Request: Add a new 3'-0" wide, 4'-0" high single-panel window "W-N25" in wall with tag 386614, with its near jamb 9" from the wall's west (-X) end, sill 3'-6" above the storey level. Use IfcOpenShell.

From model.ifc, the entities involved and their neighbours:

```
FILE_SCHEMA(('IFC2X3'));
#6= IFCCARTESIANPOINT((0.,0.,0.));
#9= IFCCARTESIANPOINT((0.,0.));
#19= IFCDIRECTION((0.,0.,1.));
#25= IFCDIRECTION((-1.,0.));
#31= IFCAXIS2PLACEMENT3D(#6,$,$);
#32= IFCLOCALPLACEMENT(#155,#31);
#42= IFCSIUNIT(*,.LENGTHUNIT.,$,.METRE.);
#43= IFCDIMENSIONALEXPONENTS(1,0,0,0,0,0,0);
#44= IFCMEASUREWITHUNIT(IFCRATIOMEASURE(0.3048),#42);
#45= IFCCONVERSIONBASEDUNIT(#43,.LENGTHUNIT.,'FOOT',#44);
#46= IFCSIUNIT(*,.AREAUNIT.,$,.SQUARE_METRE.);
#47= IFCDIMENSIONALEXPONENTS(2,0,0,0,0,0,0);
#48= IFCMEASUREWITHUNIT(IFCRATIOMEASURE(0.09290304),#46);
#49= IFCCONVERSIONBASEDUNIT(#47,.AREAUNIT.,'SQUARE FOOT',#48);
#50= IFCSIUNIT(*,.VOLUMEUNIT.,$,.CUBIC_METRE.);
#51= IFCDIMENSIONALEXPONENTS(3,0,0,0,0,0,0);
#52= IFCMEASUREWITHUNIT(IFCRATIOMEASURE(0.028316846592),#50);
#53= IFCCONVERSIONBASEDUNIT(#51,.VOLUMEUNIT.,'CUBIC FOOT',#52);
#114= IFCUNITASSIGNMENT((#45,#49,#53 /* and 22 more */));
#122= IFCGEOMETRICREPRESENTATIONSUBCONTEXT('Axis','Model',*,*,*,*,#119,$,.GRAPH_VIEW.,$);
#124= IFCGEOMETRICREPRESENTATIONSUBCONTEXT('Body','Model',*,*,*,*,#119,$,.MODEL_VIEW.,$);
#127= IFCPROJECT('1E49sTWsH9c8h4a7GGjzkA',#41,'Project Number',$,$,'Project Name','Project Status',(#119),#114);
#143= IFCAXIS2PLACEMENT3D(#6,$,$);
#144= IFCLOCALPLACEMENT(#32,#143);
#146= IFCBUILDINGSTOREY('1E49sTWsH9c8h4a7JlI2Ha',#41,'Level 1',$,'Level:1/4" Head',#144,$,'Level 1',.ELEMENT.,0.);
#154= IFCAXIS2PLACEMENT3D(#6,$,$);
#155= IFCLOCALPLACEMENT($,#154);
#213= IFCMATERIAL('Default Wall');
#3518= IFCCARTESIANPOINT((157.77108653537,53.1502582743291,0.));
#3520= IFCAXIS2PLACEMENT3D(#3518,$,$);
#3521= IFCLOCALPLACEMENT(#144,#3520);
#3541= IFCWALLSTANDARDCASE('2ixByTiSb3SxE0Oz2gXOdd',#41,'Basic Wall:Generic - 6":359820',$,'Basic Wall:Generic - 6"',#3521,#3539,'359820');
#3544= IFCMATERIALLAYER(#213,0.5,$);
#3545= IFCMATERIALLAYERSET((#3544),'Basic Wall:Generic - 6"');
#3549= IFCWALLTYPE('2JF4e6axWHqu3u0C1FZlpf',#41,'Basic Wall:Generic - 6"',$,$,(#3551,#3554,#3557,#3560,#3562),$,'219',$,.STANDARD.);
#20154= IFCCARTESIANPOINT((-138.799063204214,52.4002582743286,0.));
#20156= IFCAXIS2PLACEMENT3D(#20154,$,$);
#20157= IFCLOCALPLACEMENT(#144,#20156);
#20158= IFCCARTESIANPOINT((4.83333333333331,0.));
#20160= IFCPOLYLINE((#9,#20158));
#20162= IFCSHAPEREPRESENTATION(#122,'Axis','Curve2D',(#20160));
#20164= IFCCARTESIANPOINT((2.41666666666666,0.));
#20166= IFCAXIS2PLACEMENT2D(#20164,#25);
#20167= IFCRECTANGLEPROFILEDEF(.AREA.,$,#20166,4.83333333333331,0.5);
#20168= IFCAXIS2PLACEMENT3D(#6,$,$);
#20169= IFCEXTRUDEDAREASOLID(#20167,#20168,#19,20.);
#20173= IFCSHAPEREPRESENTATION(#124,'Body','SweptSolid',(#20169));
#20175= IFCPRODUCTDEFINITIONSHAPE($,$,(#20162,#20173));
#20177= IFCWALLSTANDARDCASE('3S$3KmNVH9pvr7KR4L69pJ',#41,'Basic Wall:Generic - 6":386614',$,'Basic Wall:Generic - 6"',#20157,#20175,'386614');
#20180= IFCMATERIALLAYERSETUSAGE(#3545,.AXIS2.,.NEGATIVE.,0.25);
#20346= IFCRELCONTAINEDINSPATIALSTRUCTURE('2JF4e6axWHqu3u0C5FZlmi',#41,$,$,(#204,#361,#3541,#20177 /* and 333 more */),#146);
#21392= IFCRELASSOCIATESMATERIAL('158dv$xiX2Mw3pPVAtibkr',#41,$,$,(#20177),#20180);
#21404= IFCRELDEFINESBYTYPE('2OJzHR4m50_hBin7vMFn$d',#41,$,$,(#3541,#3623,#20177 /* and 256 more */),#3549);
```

```python
import numpy as np
import ifcopenshell
import ifcopenshell.api.feature
import ifcopenshell.api.geometry
import ifcopenshell.api.root
import ifcopenshell.api.spatial
import ifcopenshell.api.type
import ifcopenshell.geom
import ifcopenshell.util.element
import ifcopenshell.util.placement
import ifcopenshell.util.representation
import ifcopenshell.util.shape
import ifcopenshell.util.unit

model = ifcopenshell.open("model.ifc")
unit_scale = ifcopenshell.util.unit.calculate_unit_scale(model)
settings = ifcopenshell.geom.settings()


def volume(element):
    """Net volume in cubic metres, openings subtracted."""
    shape = ifcopenshell.geom.create_shape(settings, element)
    return ifcopenshell.util.shape.get_volume(shape.geometry)


wall = model.by_guid("3S$3KmNVH9pvr7KR4L69pJ")
storey = ifcopenshell.util.element.get_container(wall, ifc_class="IfcBuildingStorey")
context = ifcopenshell.util.representation.get_context(model, "Model", "Body", "MODEL_VIEW")
before = volume(wall)

width, height, from_end, sill = 0.9144, 1.2192, 0.2286, 1.0668  # metres

# The wall runs along its own X axis, and the end named is its -X end.
wall_shape = ifcopenshell.geom.create_shape(settings, wall)
x, y, z = ifcopenshell.util.shape.get_vertices(wall_shape.geometry).T
start = x.min() + from_end
face, thickness = float(y.min()), float(y.max() - y.min())
wall_matrix = ifcopenshell.util.placement.get_local_placement(wall.ObjectPlacement)
level = ifcopenshell.util.placement.get_local_placement(storey.ObjectPlacement)[2, 3]


def in_wall(x, y):
    """Placement at x, y metres in the wall's axes, at sill height."""
    matrix = wall_matrix.copy()
    matrix[:, 3] = wall_matrix @ np.array([x / unit_scale, y / unit_scale, 0.0, 1.0])
    matrix[2, 3] = level + sill / unit_scale
    return matrix


# Opening: a box that overshoots both wall faces by 50 mm.
opening = ifcopenshell.api.root.create_entity(model, ifc_class="IfcOpeningElement")
box = ifcopenshell.api.geometry.add_wall_representation(
    model, context=context, length=width, height=height, thickness=thickness + 0.1
)
ifcopenshell.api.geometry.assign_representation(model, product=opening, representation=box)
ifcopenshell.api.geometry.edit_object_placement(model, product=opening, matrix=in_wall(start, face - 0.05), is_si=False)
ifcopenshell.api.feature.add_feature(model, feature=opening, element=wall)

window = ifcopenshell.api.root.create_entity(model, ifc_class="IfcWindow", name="W-N25")
window.OverallWidth, window.OverallHeight = width / unit_scale, height / unit_scale
body = ifcopenshell.api.geometry.add_window_representation(
    model,
    context=context,
    overall_width=window.OverallWidth,
    overall_height=window.OverallHeight,
    partition_type="SINGLE_PANEL",
)
ifcopenshell.api.geometry.assign_representation(model, product=window, representation=body)
ifcopenshell.api.spatial.assign_container(model, products=[window], relating_structure=storey)
fills = ifcopenshell.api.feature.add_filling(model, opening=opening, element=window)
fills.OwnerHistory = window.OwnerHistory  # required in IFC2X3

# IFC2X3 keeps the operation on the window style.
style = ifcopenshell.api.root.create_entity(model, ifc_class="IfcWindowStyle", name="W-N25")
style.OperationType, style.ConstructionType = "SINGLE_PANEL", "NOTDEFINED"
style.ParameterTakesPrecedence = style.Sizeable = False
ifcopenshell.api.type.assign_type(model, related_objects=[window], relating_type=style)

# Centre the window in the wall's thickness.
ifcopenshell.api.geometry.edit_object_placement(model, product=window, matrix=in_wall(start, face), is_si=False)
window_shape = ifcopenshell.geom.create_shape(settings, window)
depth = ifcopenshell.util.shape.get_vertices(window_shape.geometry)[:, 1]
offset = face + thickness / 2 - (depth.min() + depth.max()) / 2
ifcopenshell.api.geometry.edit_object_placement(model, product=window, matrix=in_wall(start, offset), is_si=False)

after = volume(wall)

print(f"wall volume {before:.3f} -> {after:.3f} m3")

model.write("model-out.ifc")
```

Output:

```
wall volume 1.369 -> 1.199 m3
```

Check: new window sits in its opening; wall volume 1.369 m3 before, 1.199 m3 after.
